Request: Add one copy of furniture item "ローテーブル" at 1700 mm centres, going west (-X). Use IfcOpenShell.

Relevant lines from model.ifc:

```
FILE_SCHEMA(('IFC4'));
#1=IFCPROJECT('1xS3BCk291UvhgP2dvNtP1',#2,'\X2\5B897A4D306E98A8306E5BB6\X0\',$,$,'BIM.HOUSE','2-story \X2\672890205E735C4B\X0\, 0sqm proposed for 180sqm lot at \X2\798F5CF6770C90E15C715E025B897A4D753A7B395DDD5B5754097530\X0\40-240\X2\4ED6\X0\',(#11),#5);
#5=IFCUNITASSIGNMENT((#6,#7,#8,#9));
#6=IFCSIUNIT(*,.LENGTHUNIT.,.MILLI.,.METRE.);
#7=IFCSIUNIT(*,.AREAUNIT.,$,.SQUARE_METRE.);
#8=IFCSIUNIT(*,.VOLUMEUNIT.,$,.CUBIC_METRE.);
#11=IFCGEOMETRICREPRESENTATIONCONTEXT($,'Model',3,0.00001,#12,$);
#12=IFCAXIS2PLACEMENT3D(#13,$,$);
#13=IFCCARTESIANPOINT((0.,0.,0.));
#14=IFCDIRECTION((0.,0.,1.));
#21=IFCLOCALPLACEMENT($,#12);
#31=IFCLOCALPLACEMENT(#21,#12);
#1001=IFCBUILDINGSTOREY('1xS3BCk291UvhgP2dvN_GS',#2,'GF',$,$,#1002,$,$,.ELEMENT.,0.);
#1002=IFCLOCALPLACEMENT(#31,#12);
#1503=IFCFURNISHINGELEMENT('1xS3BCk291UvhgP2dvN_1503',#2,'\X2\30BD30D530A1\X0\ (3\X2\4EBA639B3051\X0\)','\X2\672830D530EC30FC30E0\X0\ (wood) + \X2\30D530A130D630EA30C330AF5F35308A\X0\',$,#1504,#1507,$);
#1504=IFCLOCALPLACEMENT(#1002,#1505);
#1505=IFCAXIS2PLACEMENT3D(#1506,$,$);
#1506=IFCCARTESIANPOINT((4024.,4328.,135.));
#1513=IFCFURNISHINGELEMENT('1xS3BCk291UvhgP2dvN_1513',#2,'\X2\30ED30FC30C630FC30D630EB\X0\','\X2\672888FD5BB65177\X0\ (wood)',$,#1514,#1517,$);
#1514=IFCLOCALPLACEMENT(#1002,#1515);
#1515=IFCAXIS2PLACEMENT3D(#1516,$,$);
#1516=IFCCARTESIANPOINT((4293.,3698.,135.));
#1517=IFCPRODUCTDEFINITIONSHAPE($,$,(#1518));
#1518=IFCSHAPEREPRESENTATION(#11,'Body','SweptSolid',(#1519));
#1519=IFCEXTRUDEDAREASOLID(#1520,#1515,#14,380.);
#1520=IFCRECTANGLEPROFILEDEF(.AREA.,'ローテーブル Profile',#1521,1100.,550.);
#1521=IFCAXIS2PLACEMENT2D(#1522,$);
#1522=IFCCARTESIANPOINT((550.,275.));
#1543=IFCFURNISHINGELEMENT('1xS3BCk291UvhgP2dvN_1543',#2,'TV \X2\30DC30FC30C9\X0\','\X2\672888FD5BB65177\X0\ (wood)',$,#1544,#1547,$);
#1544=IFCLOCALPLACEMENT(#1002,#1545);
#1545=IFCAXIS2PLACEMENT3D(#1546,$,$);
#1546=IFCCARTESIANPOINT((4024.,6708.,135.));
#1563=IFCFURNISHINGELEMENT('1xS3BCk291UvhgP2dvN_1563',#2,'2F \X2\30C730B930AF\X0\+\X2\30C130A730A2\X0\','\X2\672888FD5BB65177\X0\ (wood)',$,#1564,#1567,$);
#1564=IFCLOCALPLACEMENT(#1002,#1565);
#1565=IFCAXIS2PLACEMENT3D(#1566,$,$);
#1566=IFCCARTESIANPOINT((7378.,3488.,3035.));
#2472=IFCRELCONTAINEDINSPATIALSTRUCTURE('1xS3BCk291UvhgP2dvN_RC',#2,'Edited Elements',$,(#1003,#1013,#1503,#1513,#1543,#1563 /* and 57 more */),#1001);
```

```python
import numpy as np
import ifcopenshell
import ifcopenshell.api.geometry
import ifcopenshell.api.root
import ifcopenshell.util.element
import ifcopenshell.util.placement
import ifcopenshell.util.unit

model = ifcopenshell.open("model.ifc")
unit_scale = ifcopenshell.util.unit.calculate_unit_scale(model)


def reuse_history(source, copy):
    """copy_class also copies each property set's owner history, people and application; keep the originals."""
    for rel in copy.IsDefinedBy:
        if rel.is_a("IfcRelDefinesByProperties") and (history := rel.RelatingPropertyDefinition.OwnerHistory):
            rel.RelatingPropertyDefinition.OwnerHistory = source.OwnerHistory
            ifcopenshell.util.element.remove_deep2(model, history)


source = model.by_id(1513)
base = ifcopenshell.util.placement.get_local_placement(source.ObjectPlacement)
step = np.array([-1.0, 0.0, 0.0]) * 1.7 / unit_scale

for i in range(1, 2):
    copy = ifcopenshell.api.root.copy_class(model, product=source)
    copy.Representation = ifcopenshell.util.element.copy_deep(
        model, source.Representation, exclude=["IfcGeometricRepresentationContext", "IfcRepresentationMap"]
    )
    reuse_history(source, copy)
    matrix = base.copy()
    matrix[:3, 3] += i * step
    print("added at", matrix[:3, 3].round(3) + 0.0)
    ifcopenshell.api.geometry.edit_object_placement(model, product=copy, matrix=matrix, is_si=False)

model.write("model_rev.ifc")
```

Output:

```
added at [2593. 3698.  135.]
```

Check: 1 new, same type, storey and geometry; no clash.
